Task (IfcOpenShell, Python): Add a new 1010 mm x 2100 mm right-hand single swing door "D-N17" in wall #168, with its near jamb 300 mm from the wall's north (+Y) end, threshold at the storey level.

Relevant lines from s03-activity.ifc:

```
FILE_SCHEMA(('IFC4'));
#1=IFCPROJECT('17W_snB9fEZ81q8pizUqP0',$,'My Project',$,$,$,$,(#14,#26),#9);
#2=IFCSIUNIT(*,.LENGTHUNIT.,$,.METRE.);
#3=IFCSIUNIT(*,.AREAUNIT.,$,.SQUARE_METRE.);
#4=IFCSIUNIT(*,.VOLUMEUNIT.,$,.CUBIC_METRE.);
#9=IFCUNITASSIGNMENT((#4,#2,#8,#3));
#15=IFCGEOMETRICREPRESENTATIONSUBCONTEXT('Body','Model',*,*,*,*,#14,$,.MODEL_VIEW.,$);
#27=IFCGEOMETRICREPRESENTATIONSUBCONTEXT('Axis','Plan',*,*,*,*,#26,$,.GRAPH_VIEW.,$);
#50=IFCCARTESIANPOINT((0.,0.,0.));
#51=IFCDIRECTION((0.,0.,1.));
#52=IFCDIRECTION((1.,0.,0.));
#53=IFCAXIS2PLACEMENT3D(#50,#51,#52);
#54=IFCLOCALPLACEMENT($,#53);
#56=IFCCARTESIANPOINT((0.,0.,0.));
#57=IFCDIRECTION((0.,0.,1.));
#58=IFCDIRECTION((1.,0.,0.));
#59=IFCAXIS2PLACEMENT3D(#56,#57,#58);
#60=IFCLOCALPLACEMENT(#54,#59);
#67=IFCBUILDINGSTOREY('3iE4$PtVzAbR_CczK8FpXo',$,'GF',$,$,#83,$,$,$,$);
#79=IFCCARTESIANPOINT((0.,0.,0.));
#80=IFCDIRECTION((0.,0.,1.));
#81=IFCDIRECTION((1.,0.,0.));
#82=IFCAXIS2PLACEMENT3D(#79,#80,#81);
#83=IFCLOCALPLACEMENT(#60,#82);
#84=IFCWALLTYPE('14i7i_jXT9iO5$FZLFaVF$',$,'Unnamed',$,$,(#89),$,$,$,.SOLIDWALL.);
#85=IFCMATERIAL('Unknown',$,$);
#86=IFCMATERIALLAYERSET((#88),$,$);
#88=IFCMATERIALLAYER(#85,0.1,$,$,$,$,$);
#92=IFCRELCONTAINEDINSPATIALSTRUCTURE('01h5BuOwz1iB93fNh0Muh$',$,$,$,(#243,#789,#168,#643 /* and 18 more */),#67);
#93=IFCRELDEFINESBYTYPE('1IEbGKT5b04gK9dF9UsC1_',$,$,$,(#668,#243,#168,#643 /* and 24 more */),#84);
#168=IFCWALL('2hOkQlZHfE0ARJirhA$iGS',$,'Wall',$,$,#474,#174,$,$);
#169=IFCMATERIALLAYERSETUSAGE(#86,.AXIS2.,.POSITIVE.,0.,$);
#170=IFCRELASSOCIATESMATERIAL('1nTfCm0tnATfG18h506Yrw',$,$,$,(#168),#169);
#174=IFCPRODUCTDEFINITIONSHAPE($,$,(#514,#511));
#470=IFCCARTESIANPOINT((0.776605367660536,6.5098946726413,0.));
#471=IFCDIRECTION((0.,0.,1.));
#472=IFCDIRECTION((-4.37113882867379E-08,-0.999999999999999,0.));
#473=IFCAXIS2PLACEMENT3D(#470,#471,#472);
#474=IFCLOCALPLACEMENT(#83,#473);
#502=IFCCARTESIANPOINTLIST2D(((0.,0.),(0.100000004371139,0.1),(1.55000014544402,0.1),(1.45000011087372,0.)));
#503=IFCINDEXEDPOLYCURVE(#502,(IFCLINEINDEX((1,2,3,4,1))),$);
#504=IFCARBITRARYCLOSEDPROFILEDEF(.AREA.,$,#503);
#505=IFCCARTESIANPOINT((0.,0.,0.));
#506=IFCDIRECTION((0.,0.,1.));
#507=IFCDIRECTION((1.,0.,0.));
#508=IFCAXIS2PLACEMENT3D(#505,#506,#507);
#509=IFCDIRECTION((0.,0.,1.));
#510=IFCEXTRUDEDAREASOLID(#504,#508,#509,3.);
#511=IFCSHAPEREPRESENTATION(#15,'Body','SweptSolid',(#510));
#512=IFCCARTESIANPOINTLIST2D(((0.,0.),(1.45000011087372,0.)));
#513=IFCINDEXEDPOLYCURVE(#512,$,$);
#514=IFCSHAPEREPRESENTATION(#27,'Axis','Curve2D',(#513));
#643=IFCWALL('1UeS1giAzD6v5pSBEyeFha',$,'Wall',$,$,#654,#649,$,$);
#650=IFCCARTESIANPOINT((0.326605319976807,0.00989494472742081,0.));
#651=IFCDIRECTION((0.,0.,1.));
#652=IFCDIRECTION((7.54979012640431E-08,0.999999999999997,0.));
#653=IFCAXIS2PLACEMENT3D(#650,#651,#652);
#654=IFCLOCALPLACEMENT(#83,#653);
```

```python
import numpy as np
import ifcopenshell
import ifcopenshell.api.feature
import ifcopenshell.api.geometry
import ifcopenshell.api.root
import ifcopenshell.api.spatial
import ifcopenshell.geom
import ifcopenshell.util.element
import ifcopenshell.util.placement
import ifcopenshell.util.representation
import ifcopenshell.util.shape
import ifcopenshell.util.unit

model = ifcopenshell.open("s03-activity.ifc")
unit_scale = ifcopenshell.util.unit.calculate_unit_scale(model)
settings = ifcopenshell.geom.settings()


def volume(element):
    """Net volume in cubic metres, openings subtracted."""
    shape = ifcopenshell.geom.create_shape(settings, element)
    return ifcopenshell.util.shape.get_volume(shape.geometry)


wall = model.by_guid("2hOkQlZHfE0ARJirhA$iGS")
storey = ifcopenshell.util.element.get_container(wall, ifc_class="IfcBuildingStorey")
context = ifcopenshell.util.representation.get_context(model, "Model", "Body", "MODEL_VIEW")
before = volume(wall)

width, height, from_end, sill = 1.01, 2.1, 0.3, 0.0  # metres

# The wall runs along its own X axis, and the end named is its -X end.
wall_shape = ifcopenshell.geom.create_shape(settings, wall)
x, y, z = ifcopenshell.util.shape.get_vertices(wall_shape.geometry).T
start = x.min() + from_end
face, thickness = float(y.min()), float(y.max() - y.min())
wall_matrix = ifcopenshell.util.placement.get_local_placement(wall.ObjectPlacement)
level = ifcopenshell.util.placement.get_local_placement(storey.ObjectPlacement)[2, 3]


def in_wall(x, y):
    """Placement at x, y metres in the wall's axes, at sill height."""
    matrix = wall_matrix.copy()
    matrix[:, 3] = wall_matrix @ np.array([x / unit_scale, y / unit_scale, 0.0, 1.0])
    matrix[2, 3] = level + sill / unit_scale
    return matrix


# Opening: a box that overshoots both wall faces by 50 mm.
opening = ifcopenshell.api.root.create_entity(model, ifc_class="IfcOpeningElement", predefined_type="OPENING")
box = ifcopenshell.api.geometry.add_wall_representation(
    model, context=context, length=width, height=height, thickness=thickness + 0.1
)
ifcopenshell.api.geometry.assign_representation(model, product=opening, representation=box)
ifcopenshell.api.geometry.edit_object_placement(model, product=opening, matrix=in_wall(start, face - 0.05), is_si=False)
ifcopenshell.api.feature.add_feature(model, feature=opening, element=wall)

door = ifcopenshell.api.root.create_entity(model, ifc_class="IfcDoor", name="D-N17", predefined_type="DOOR")
door.OverallWidth, door.OverallHeight = width / unit_scale, height / unit_scale
door.OperationType = "SINGLE_SWING_RIGHT"
body = ifcopenshell.api.geometry.add_door_representation(
    model,
    context=context,
    overall_width=door.OverallWidth,
    overall_height=door.OverallHeight,
    operation_type="SINGLE_SWING_RIGHT",
    lining_properties={"LiningDepth": thickness / unit_scale, "ThresholdDepth": thickness / unit_scale},
)
ifcopenshell.api.geometry.assign_representation(model, product=door, representation=body)
ifcopenshell.api.spatial.assign_container(model, products=[door], relating_structure=storey)
ifcopenshell.api.feature.add_filling(model, opening=opening, element=door)

# The lining spans the wall, so the door starts at the wall face.
ifcopenshell.api.geometry.edit_object_placement(model, product=door, matrix=in_wall(start, face), is_si=False)

after = volume(wall)

print(f"wall volume {before:.3f} -> {after:.3f} m3")

model.write("s03-activity_updated.ifc")
```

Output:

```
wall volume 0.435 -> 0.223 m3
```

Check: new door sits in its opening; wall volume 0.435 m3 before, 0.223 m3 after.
